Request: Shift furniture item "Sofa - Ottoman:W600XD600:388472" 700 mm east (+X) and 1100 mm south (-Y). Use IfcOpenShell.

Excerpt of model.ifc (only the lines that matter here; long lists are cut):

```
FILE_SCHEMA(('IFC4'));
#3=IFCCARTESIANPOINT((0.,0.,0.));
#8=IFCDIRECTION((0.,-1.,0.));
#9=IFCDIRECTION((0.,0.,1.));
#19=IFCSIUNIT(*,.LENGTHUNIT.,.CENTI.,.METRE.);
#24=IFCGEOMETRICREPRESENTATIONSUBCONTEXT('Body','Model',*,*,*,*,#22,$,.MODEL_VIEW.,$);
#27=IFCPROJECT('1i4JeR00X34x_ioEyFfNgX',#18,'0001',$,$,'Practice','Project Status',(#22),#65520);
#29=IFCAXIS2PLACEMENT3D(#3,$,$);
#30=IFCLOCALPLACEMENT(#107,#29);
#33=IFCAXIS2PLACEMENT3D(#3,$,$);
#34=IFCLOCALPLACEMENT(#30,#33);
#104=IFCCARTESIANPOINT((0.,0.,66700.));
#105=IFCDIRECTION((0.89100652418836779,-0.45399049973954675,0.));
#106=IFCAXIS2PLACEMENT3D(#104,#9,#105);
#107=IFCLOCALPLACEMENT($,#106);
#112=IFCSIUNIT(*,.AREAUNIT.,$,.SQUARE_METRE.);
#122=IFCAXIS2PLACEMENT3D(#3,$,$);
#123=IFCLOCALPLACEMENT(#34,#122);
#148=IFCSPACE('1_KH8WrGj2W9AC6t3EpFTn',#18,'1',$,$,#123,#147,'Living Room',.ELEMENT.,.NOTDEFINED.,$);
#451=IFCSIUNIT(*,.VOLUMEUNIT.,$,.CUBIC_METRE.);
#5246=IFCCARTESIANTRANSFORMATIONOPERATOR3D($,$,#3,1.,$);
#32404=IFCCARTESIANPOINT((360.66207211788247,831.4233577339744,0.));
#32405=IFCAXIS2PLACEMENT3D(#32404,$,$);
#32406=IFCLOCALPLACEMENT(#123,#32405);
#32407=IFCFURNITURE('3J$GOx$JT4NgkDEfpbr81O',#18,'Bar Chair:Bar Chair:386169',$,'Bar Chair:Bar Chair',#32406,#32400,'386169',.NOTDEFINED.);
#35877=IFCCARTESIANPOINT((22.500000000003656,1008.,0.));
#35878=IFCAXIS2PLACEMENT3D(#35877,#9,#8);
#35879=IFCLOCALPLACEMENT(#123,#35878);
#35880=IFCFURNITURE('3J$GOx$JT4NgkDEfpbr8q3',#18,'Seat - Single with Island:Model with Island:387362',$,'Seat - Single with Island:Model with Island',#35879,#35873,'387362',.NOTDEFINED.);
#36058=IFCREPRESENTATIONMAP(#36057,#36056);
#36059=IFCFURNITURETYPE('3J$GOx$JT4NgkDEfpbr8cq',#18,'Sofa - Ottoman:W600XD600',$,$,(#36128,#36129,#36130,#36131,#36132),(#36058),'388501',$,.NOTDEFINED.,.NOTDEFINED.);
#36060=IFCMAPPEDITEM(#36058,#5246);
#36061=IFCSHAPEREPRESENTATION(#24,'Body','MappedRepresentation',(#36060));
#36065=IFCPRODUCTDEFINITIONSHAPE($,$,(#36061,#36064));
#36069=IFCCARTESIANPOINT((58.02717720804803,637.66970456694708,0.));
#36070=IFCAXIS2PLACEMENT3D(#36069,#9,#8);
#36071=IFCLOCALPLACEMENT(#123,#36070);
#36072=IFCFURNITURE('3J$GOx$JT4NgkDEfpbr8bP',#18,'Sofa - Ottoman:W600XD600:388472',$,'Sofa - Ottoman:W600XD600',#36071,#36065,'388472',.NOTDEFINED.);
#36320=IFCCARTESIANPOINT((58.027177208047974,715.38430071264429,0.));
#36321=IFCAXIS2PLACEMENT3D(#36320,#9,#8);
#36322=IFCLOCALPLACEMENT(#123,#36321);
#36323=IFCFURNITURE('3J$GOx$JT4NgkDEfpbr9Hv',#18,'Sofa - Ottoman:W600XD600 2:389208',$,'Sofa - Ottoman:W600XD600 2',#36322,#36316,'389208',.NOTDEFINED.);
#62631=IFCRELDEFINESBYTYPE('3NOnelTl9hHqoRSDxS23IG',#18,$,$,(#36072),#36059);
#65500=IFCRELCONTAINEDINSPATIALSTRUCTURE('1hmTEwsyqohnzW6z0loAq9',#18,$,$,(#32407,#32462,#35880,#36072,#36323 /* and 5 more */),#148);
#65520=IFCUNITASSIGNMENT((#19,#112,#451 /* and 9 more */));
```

```python
import ifcopenshell
import ifcopenshell.api.geometry
import ifcopenshell.util.placement
import ifcopenshell.util.unit

model = ifcopenshell.open("model.ifc")
unit_scale = ifcopenshell.util.unit.calculate_unit_scale(model)

item = model.by_guid("3J$GOx$JT4NgkDEfpbr8bP")
matrix = ifcopenshell.util.placement.get_local_placement(item.ObjectPlacement)
matrix[0, 3] += 0.7 / unit_scale
matrix[1, 3] -= 1.1 / unit_scale
ifcopenshell.api.geometry.edit_object_placement(model, product=item, matrix=matrix, is_si=False)

print(ifcopenshell.util.placement.get_local_placement(item.ObjectPlacement).round(3) + 0.0)

model.write("model_v2.ifc")
```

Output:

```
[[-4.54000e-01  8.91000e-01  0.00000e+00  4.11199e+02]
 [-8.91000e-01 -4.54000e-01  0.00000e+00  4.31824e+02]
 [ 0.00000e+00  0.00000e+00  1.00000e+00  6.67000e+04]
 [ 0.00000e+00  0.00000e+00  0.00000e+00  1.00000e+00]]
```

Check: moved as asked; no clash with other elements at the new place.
